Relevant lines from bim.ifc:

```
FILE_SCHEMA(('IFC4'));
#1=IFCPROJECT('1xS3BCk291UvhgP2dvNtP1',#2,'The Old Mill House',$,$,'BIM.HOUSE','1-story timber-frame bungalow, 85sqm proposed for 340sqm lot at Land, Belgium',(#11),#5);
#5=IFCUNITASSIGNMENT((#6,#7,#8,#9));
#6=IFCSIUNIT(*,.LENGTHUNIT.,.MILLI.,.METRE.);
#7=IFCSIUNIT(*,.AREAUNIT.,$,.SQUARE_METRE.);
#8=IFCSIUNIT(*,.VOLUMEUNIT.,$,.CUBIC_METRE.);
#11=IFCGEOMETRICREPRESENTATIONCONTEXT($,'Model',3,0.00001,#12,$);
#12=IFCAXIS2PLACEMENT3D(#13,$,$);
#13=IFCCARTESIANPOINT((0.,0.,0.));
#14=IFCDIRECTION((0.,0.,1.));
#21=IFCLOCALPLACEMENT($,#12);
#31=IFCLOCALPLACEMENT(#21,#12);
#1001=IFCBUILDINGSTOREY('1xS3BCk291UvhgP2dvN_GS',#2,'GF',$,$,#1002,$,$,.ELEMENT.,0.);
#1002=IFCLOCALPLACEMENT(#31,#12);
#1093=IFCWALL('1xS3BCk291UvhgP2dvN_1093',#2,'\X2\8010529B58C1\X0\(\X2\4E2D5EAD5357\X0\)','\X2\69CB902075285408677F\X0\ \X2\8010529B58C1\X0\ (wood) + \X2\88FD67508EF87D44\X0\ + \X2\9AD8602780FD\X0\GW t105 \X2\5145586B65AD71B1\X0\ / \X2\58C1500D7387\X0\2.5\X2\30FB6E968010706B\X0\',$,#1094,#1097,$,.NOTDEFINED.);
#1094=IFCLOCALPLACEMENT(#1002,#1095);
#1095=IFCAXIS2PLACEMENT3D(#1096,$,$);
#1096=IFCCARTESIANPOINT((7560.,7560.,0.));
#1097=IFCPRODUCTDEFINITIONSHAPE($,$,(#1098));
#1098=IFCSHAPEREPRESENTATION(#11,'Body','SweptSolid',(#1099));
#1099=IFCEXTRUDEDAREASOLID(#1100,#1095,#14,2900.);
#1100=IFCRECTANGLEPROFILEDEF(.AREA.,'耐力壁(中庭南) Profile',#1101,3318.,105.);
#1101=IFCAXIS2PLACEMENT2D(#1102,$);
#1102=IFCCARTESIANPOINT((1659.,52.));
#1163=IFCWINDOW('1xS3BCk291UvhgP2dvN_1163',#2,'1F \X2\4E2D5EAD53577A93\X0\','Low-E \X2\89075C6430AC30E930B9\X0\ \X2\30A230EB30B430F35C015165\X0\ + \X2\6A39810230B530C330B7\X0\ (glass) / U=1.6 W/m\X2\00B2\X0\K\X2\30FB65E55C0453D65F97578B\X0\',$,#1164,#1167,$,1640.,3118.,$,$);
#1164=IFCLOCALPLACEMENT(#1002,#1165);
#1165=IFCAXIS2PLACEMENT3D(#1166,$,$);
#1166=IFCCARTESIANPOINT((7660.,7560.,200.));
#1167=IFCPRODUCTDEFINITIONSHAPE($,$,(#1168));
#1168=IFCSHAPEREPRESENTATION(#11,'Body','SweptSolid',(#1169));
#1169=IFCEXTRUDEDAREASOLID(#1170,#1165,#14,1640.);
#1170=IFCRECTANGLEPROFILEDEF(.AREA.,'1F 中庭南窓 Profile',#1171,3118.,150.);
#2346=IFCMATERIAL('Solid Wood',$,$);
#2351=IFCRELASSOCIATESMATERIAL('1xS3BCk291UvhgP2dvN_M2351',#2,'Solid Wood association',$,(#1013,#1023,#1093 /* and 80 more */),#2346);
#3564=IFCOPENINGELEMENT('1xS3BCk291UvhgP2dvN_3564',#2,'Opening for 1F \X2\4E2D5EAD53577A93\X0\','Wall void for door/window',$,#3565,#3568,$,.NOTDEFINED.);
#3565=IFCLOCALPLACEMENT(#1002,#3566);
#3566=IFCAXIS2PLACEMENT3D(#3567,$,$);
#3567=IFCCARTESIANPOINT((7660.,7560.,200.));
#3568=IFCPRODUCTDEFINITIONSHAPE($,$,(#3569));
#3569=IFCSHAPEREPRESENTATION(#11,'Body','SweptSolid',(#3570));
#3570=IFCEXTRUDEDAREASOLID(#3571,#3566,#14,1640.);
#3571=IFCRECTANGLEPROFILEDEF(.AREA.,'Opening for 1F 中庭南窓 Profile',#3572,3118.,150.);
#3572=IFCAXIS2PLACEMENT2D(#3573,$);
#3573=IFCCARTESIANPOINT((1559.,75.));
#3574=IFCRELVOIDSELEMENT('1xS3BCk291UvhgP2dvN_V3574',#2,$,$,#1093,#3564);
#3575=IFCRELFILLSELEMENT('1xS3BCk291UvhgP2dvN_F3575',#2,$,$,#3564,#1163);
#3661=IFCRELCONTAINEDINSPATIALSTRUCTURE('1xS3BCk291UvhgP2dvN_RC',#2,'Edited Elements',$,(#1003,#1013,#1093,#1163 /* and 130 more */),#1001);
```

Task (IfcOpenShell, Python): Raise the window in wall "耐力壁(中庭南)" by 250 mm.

```python
import numpy as np
import ifcopenshell
import ifcopenshell.api.geometry
import ifcopenshell.util.placement
import ifcopenshell.util.unit

model = ifcopenshell.open("bim.ifc")
unit_scale = ifcopenshell.util.unit.calculate_unit_scale(model)

window = model.by_id(1163)
opening = window.FillsVoids[0].RelatingOpeningElement
dz = 0.25 / unit_scale

shift = np.array([0.0, 0.0, dz])
# The window is not placed relative to its opening, so move both.
for product in (opening, window):
    matrix = ifcopenshell.util.placement.get_local_placement(product.ObjectPlacement)
    matrix[:3, 3] += shift
    ifcopenshell.api.geometry.edit_object_placement(model, product=product, matrix=matrix, is_si=False)

print(f"moved by {dz * unit_scale:+.3f} m")

model.write("bim_v2.ifc")
```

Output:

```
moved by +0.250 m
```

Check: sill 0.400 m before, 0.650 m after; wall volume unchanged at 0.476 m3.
